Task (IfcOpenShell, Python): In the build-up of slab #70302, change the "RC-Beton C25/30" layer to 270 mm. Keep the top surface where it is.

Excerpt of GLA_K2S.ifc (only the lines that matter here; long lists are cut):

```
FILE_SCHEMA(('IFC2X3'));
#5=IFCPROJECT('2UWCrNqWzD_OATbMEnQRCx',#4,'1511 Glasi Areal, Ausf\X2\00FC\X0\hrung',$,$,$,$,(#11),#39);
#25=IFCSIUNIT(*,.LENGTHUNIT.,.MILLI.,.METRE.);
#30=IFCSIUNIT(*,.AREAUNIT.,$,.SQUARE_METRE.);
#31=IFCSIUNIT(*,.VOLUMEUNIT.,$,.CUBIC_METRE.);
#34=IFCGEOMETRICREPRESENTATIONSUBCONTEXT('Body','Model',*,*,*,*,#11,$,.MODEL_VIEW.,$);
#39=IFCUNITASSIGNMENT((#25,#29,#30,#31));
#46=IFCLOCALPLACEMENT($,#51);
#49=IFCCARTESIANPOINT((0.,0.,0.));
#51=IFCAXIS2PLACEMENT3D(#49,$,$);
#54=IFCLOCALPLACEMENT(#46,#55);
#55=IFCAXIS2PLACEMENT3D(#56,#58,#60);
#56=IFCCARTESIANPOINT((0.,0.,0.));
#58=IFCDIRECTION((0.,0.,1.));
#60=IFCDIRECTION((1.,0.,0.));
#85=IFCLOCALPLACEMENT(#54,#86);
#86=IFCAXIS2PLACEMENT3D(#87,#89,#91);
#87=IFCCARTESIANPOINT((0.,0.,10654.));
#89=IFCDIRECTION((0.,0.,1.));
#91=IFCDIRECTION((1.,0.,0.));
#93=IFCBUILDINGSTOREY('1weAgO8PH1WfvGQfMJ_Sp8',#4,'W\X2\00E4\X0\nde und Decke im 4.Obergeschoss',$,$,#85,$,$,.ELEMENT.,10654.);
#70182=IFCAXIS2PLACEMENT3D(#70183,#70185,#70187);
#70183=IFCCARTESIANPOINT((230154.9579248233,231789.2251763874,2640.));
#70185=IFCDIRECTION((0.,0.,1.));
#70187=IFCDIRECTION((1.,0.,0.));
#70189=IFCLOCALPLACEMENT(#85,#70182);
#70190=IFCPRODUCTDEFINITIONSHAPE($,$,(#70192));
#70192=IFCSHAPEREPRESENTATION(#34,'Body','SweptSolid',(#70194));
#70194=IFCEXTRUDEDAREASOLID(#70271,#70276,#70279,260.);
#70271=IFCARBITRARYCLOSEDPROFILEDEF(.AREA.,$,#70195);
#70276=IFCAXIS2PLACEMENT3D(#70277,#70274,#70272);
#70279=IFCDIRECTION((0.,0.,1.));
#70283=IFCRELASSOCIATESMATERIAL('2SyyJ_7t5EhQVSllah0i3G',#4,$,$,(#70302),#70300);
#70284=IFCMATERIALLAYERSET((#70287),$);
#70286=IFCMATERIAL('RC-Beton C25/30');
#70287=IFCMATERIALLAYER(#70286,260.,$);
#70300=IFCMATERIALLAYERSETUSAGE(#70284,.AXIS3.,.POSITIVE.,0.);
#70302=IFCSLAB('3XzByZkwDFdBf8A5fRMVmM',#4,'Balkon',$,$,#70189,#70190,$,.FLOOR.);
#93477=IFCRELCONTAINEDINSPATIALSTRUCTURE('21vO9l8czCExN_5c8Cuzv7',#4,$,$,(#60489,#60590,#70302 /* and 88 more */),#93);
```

```python
import ifcopenshell
import ifcopenshell.util.element
import ifcopenshell.util.representation

model = ifcopenshell.open("GLA_K2S.ifc")

layer_set = model.by_id(70284)
layer = next(l for l in layer_set.MaterialLayers if l.Material and l.Material.Name == "RC-Beton C25/30")
change = 270.0 - layer.LayerThickness
layer.LayerThickness += change

# Geometry does not follow the layer set by itself.
slabs = [e for e in ifcopenshell.util.element.get_elements_by_material(model, layer_set) if e.is_a("IfcSlab")]
for slab in sorted(slabs, key=lambda e: e.id()):
    body = ifcopenshell.util.representation.get_representation(slab, "Model", "Body")
    solid = body.Items[0]
    old_depth = solid.Depth
    solid.Depth += change
    # Extruded upwards: lower the start of the extrusion so the top stays.
    x, y, z = solid.Position.Location.Coordinates
    solid.Position.Location = model.createIfcCartesianPoint((x, y, z - change))
    print(slab.id(), f"{old_depth:g} -> {solid.Depth:g}")

# The layers are counted up from the underside, which has moved.
for usage in {ifcopenshell.util.element.get_material(slab) for slab in slabs}:
    usage.OffsetFromReferenceLine -= change

model.write("GLA_K2S_rev.ifc")
```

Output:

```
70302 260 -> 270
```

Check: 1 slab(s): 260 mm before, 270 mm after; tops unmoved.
